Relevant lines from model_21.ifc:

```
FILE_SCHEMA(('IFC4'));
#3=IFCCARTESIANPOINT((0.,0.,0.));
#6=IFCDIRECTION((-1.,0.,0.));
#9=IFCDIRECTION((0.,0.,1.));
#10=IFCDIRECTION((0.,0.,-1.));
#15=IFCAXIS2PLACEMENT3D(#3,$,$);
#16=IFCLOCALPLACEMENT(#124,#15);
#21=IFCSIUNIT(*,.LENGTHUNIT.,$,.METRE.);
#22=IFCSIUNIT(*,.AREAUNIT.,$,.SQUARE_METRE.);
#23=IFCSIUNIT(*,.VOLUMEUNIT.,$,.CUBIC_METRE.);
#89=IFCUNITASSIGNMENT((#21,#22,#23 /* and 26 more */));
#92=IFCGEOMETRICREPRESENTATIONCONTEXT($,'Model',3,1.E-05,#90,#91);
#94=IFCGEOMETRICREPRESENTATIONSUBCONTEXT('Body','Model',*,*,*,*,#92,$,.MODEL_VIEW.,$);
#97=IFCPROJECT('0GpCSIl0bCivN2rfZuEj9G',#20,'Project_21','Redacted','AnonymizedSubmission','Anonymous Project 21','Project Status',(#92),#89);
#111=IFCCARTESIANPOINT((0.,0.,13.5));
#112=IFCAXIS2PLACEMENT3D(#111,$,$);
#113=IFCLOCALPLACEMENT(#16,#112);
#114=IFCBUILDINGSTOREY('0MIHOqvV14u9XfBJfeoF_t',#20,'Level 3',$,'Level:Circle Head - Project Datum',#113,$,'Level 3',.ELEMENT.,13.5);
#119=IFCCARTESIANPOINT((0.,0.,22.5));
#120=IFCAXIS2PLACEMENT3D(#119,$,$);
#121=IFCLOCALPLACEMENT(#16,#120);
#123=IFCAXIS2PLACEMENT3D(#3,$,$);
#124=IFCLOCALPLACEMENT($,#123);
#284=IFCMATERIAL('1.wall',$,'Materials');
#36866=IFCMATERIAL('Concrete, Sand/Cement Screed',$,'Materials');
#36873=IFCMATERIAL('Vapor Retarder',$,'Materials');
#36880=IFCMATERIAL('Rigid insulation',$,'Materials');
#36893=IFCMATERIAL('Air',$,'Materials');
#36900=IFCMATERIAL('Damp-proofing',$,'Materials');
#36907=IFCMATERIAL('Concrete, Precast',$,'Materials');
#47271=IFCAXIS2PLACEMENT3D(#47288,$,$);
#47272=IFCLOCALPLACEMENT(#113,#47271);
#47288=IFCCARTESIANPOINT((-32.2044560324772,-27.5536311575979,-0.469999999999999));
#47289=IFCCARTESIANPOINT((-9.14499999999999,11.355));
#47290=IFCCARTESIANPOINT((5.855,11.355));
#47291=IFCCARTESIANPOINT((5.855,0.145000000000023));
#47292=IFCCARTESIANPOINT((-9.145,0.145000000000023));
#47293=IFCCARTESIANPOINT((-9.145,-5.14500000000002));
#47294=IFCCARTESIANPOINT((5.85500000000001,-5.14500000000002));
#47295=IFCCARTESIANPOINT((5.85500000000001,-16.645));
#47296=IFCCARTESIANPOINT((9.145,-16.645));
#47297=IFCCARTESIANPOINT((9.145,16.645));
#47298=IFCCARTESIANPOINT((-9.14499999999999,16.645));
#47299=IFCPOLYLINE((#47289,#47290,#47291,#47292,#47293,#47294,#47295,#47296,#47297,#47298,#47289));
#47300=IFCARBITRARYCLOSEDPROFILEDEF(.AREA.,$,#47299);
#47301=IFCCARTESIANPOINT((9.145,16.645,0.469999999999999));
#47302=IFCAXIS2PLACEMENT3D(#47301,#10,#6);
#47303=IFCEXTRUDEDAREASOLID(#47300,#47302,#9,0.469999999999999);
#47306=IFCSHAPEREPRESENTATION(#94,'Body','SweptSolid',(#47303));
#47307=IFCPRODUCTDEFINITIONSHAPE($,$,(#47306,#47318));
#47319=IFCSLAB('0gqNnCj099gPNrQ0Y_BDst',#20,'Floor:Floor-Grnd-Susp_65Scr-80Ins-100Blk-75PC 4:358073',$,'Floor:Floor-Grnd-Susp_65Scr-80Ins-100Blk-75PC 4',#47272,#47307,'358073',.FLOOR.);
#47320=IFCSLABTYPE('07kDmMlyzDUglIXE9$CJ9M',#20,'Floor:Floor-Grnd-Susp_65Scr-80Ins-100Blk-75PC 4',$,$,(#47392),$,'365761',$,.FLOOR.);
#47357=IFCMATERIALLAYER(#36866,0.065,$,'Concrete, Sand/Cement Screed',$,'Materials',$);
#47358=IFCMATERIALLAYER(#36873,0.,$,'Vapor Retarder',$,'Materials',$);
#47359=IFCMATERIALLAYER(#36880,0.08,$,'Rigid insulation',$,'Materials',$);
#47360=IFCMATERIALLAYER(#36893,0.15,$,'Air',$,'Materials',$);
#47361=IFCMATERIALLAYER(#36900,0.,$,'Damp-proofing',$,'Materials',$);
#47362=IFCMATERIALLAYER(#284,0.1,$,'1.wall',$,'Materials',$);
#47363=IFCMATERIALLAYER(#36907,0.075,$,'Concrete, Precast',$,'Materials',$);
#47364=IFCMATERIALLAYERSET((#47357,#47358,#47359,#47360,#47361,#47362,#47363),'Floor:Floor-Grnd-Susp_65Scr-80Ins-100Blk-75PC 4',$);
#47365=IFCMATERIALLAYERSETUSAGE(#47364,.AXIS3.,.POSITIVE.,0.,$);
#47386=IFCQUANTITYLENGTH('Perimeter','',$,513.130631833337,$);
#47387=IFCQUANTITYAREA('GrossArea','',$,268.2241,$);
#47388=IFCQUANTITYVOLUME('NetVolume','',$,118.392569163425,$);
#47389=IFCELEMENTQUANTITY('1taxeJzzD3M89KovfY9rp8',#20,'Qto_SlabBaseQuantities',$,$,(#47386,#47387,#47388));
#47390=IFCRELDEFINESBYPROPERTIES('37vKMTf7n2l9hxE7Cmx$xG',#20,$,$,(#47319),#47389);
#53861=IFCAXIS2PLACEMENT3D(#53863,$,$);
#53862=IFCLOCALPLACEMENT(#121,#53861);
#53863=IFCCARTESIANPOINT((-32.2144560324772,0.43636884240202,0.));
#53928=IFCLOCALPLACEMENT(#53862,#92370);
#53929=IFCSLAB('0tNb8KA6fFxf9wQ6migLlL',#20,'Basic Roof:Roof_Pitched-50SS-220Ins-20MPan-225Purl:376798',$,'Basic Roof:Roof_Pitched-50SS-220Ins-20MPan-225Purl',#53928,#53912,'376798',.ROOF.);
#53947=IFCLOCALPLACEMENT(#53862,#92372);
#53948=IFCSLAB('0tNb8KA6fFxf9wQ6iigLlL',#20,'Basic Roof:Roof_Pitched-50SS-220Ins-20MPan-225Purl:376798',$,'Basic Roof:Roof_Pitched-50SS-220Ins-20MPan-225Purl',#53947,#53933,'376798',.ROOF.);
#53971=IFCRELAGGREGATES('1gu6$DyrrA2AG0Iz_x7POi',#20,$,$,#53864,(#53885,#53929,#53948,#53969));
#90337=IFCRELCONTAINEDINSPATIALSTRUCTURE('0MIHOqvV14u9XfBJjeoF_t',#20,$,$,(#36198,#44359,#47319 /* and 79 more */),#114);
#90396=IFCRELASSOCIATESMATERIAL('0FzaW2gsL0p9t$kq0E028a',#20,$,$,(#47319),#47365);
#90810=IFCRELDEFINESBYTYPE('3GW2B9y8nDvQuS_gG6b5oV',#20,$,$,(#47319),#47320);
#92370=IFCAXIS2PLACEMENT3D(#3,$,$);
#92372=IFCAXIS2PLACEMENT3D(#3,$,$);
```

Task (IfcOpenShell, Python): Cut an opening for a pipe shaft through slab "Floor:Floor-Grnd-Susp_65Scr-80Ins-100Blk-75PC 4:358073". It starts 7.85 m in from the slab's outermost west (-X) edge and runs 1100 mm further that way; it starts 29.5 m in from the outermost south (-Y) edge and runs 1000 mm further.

```python
import numpy as np
import ifcopenshell
import ifcopenshell.api.feature
import ifcopenshell.api.geometry
import ifcopenshell.api.pset
import ifcopenshell.api.root
import ifcopenshell.geom
import ifcopenshell.util.element
import ifcopenshell.util.placement
import ifcopenshell.util.representation
import ifcopenshell.util.shape
import ifcopenshell.util.unit

model = ifcopenshell.open("model_21.ifc")
unit_scale = ifcopenshell.util.unit.calculate_unit_scale(model)
volume_scale = ifcopenshell.util.unit.calculate_unit_scale(model, "VOLUMEUNIT")
settings = ifcopenshell.geom.settings()


def volume(element):
    """Net volume in cubic metres, openings subtracted."""
    shape = ifcopenshell.geom.create_shape(settings, element)
    return ifcopenshell.util.shape.get_volume(shape.geometry)


slab = model.by_guid("0gqNnCj099gPNrQ0Y_BDst")
before = volume(slab)

# Extent in the slab's own axes, in metres. The edges named are its -X and -Y sides.
slab_shape = ifcopenshell.geom.create_shape(settings, slab)
vertices = ifcopenshell.util.shape.get_vertices(slab_shape.geometry)
x_min, y_min, bottom = vertices.min(axis=0)
top = vertices[:, 2].max()

opening = ifcopenshell.api.root.create_entity(model, ifc_class="IfcOpeningElement", name="Pipe shaft opening", predefined_type="OPENING")
context = ifcopenshell.util.representation.get_context(model, "Model", "Body", "MODEL_VIEW")
width, depth = 1.1, 1
outline = [(0.0, 0.0), (width, 0.0), (width, depth), (0.0, depth), (0.0, 0.0)]
# Overshoot both faces by 50 mm so the cut is clean.
shape = ifcopenshell.api.geometry.add_slab_representation(
    model, context=context, depth=top - bottom + 0.1, polyline=outline
)
ifcopenshell.api.geometry.assign_representation(model, product=opening, representation=shape)

matrix = ifcopenshell.util.placement.get_local_placement(slab.ObjectPlacement)
matrix[:, 3] = matrix @ np.append(np.array([x_min + 7.85, y_min + 29.5, bottom - 0.05]) / unit_scale, 1.0)
ifcopenshell.api.geometry.edit_object_placement(model, product=opening, matrix=matrix, is_si=False)
ifcopenshell.api.feature.add_feature(model, feature=opening, element=slab)

after = volume(slab)

# Update the slab's stored quantities.
qto = model.by_id(ifcopenshell.util.element.get_pset(slab, "Qto_SlabBaseQuantities", should_inherit=False)["id"])
ifcopenshell.api.pset.edit_qto(model, qto=qto, properties={"NetVolume": after / volume_scale})

print(f"slab volume {before:.3f} -> {after:.3f} m3")

model.write("model_21_edited.ifc")
```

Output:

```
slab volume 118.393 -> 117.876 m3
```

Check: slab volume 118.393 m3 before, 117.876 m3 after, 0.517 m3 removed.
